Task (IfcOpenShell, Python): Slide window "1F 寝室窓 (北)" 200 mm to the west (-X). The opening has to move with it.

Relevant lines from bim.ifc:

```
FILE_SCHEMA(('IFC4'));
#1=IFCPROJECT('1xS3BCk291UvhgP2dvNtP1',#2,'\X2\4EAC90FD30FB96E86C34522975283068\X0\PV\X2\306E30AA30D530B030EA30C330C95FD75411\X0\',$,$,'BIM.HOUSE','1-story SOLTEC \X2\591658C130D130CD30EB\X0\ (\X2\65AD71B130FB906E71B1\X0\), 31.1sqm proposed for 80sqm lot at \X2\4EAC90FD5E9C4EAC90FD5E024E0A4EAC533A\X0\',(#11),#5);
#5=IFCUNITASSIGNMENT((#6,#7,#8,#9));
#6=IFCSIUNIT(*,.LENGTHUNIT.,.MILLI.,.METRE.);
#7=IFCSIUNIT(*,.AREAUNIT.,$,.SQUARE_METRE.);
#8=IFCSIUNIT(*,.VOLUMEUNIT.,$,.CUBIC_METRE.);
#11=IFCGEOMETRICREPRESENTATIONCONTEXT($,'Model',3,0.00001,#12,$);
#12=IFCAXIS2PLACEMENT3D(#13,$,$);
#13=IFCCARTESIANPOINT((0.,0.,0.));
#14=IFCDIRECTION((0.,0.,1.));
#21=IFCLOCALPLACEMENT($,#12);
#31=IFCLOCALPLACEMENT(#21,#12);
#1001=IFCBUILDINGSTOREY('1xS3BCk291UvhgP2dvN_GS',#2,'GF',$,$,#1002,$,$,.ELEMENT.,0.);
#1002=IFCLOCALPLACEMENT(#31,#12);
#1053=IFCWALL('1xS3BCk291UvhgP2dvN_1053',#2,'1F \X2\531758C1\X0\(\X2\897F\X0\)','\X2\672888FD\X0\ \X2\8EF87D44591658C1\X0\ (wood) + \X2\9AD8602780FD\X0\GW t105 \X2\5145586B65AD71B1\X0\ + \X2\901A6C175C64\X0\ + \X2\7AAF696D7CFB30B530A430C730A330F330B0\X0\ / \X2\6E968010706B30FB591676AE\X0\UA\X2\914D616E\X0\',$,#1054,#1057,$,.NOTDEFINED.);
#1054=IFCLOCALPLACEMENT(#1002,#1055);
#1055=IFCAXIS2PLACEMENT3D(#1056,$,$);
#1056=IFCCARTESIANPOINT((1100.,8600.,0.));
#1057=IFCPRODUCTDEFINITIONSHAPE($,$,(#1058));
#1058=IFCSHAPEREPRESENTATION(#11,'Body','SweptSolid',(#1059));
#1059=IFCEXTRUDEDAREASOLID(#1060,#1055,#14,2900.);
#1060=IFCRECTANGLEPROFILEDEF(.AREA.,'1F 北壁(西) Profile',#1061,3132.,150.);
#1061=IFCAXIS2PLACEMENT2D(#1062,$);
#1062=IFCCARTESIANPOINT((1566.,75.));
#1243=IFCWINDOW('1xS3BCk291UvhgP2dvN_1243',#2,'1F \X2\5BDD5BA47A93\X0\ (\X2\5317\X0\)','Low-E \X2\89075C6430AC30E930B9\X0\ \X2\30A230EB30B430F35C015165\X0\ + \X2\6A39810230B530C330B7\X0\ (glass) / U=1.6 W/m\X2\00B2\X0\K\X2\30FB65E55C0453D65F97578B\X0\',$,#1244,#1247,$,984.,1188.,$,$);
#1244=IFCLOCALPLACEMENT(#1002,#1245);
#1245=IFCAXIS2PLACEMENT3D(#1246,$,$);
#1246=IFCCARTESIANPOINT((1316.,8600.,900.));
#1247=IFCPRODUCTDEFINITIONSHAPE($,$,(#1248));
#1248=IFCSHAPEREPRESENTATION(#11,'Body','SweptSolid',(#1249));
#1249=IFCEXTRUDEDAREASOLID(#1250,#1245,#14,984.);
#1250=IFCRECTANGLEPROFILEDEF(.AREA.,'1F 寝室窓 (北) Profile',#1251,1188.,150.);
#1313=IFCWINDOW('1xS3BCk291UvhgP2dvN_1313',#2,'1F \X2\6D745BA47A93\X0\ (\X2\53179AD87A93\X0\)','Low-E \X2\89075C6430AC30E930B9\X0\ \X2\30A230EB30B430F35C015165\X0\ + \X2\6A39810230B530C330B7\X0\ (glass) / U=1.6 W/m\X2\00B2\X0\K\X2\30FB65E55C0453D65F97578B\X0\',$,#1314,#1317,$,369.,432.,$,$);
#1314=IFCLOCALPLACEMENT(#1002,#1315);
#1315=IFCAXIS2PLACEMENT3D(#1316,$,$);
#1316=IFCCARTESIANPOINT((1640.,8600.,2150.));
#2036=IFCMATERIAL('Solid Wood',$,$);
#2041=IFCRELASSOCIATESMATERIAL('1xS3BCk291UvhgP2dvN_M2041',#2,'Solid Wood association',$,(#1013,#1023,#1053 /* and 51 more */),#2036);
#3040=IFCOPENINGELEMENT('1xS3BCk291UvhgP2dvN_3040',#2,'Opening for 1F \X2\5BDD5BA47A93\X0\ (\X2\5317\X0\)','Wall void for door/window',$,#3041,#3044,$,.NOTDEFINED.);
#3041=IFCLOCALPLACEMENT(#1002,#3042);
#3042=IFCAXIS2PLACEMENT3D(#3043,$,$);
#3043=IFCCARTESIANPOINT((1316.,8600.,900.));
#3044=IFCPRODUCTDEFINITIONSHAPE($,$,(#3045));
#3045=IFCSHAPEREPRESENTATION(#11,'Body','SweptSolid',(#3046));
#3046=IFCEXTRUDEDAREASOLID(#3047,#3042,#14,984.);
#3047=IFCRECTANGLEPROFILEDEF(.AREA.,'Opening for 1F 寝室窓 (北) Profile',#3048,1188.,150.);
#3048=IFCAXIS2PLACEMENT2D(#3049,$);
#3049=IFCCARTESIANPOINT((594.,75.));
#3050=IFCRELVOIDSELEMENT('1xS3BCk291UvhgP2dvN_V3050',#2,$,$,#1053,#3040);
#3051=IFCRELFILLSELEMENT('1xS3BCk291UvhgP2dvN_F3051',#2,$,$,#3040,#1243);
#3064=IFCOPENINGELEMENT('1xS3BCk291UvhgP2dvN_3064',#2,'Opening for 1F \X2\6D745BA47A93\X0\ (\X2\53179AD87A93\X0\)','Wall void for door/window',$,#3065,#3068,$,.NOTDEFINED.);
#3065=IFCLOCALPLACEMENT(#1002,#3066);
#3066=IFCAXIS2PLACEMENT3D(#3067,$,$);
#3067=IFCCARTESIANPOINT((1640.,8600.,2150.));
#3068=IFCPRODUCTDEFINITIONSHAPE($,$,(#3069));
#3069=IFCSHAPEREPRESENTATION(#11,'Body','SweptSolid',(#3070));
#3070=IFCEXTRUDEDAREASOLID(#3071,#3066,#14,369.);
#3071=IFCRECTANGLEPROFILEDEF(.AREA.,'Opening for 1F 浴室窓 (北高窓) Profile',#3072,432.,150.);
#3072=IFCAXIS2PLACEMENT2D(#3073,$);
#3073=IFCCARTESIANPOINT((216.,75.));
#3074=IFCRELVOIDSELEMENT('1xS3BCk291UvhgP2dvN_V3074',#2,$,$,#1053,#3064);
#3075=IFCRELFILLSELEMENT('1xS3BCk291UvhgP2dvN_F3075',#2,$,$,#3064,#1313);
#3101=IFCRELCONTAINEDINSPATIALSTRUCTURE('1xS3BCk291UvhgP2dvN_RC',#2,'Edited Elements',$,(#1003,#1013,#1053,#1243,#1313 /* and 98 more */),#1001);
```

```python
import ifcopenshell
import ifcopenshell.api.geometry
import ifcopenshell.util.placement

model = ifcopenshell.open("bim.ifc")

window = model.by_guid("1xS3BCk291UvhgP2dvN_1243")
opening = window.FillsVoids[0].RelatingOpeningElement
wall = opening.VoidsElements[0].RelatingBuildingElement

wall_matrix = ifcopenshell.util.placement.get_local_placement(wall.ObjectPlacement)
shift = wall_matrix[:3, 0] * -200.0
before = ifcopenshell.util.placement.get_local_placement(window.ObjectPlacement)[:3, 3].copy()

# The window is not placed relative to its opening, so move both.
for product in (opening, window):
    matrix = ifcopenshell.util.placement.get_local_placement(product.ObjectPlacement)
    matrix[:3, 3] += shift
    ifcopenshell.api.geometry.edit_object_placement(model, product=product, matrix=matrix, is_si=False)

after = ifcopenshell.util.placement.get_local_placement(window.ObjectPlacement)[:3, 3]
print("window moved by", (after - before).round(3) + 0.0)

model.write("bim-out.ifc")
```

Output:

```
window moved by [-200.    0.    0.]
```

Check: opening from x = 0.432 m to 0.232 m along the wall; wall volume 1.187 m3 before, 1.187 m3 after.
